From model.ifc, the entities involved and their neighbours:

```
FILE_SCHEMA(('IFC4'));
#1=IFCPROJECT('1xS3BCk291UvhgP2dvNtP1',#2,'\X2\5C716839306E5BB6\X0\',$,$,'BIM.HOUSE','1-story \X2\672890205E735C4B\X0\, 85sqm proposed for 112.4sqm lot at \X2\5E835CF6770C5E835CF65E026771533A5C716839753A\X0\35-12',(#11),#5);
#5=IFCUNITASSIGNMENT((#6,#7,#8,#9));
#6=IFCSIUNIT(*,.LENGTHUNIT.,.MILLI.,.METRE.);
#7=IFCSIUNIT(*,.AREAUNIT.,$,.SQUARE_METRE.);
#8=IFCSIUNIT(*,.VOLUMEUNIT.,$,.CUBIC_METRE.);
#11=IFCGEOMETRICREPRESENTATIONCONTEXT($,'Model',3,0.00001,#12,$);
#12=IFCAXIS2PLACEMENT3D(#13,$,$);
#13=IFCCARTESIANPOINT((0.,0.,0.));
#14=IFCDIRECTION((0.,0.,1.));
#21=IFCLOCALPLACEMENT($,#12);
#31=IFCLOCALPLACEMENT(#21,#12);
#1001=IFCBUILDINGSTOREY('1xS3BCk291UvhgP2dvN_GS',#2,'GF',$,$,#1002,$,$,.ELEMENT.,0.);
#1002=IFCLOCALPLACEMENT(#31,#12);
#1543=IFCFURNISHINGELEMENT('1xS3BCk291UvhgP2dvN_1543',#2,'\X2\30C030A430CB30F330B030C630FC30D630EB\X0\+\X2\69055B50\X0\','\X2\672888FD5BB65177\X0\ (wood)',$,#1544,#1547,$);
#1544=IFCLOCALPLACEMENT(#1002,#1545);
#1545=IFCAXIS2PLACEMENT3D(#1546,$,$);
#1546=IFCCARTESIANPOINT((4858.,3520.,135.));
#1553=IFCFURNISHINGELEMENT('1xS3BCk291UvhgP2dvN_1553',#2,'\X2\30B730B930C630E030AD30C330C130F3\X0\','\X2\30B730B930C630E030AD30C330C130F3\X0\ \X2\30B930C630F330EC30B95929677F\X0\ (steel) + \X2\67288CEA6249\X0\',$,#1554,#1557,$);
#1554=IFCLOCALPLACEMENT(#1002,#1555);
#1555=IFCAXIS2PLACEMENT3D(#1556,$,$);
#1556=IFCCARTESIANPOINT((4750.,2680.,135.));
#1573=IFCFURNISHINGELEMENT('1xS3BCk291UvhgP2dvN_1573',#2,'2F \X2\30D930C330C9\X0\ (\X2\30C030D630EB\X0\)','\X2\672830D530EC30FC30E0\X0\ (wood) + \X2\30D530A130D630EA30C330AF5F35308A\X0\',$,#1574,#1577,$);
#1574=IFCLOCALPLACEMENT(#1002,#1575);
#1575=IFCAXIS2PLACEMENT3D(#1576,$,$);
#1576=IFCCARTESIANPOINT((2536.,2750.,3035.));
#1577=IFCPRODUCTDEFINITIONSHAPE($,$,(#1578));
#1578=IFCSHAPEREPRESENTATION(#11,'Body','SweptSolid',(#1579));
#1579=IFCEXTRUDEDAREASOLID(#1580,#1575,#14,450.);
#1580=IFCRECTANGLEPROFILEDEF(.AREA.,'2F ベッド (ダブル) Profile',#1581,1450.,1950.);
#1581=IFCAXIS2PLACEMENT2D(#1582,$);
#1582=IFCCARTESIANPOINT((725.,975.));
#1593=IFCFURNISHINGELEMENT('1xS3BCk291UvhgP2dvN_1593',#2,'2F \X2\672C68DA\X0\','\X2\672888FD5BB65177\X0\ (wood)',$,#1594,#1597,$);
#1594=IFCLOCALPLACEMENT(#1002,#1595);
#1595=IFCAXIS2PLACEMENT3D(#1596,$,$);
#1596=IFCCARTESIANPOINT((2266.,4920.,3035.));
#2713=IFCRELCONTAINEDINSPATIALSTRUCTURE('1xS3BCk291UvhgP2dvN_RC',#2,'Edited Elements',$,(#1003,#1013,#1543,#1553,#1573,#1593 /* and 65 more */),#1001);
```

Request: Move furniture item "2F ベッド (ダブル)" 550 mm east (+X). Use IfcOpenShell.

```python
import ifcopenshell
import ifcopenshell.api.geometry
import ifcopenshell.util.placement
import ifcopenshell.util.unit

model = ifcopenshell.open("model.ifc")
unit_scale = ifcopenshell.util.unit.calculate_unit_scale(model)

item = model.by_guid("1xS3BCk291UvhgP2dvN_1573")
matrix = ifcopenshell.util.placement.get_local_placement(item.ObjectPlacement)
matrix[0, 3] += 0.55 / unit_scale
ifcopenshell.api.geometry.edit_object_placement(model, product=item, matrix=matrix, is_si=False)

print(ifcopenshell.util.placement.get_local_placement(item.ObjectPlacement).round(3) + 0.0)

model.write("model_updated.ifc")
```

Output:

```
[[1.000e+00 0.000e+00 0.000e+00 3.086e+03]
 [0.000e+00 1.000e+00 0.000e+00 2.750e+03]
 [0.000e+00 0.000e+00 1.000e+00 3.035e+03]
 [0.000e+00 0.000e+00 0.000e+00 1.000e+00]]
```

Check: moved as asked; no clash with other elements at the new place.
